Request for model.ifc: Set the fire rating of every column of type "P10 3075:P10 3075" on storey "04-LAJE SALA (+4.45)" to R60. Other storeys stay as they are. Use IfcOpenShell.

First a look at what the model holds.

```python
import ifcopenshell
import ifcopenshell.util.element

model = ifcopenshell.open("model.ifc")
print(model.schema)
storey = next(s for s in model.by_type("IfcBuildingStorey") if s.Name == "04-LAJE SALA (+4.45)")
columns = [e for e in ifcopenshell.util.element.get_decomposition(storey) if e.is_a("IfcColumn")]
seen = {}
for e in columns:
    element_type = ifcopenshell.util.element.get_type(e)
    key = (element_type.Name if element_type != e and element_type else None, ifcopenshell.util.element.get_pset(e, "Pset_ColumnCommon", "FireRating"))
    seen[key] = seen.get(key, 0) + 1
for (name, value), count in sorted(seen.items(), key=str):
    print(count, "x", name, "|", value)
```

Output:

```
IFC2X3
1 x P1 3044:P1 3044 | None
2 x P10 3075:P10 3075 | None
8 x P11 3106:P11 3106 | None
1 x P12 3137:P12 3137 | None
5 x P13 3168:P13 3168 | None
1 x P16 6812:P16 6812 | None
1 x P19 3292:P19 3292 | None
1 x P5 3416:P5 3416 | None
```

```python
import ifcopenshell
import ifcopenshell.api.pset
import ifcopenshell.util.element

model = ifcopenshell.open("model.ifc")

storey = next(s for s in model.by_type("IfcBuildingStorey") if s.Name == "04-LAJE SALA (+4.45)")
columns = [e for e in ifcopenshell.util.element.get_decomposition(storey) if e.is_a("IfcColumn")]

count = 0
for e in columns:
    element_type = ifcopenshell.util.element.get_type(e)
    if element_type in (None, e) or element_type.Name != "P10 3075:P10 3075":
        continue
    # add_pset returns the element's existing set when there is one.
    pset = ifcopenshell.api.pset.add_pset(model, product=e, name="Pset_ColumnCommon")
    ifcopenshell.api.pset.edit_pset(model, pset=pset, properties={"FireRating": "R60"})
    count += 1

print(count, "columns updated")

model.write("model_rev.ifc")
```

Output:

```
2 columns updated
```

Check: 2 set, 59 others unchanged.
